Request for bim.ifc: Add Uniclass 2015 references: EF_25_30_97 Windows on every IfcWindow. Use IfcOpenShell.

First a look at what the model holds.

```python
import ifcopenshell

model = ifcopenshell.open("bim.ifc")
print(model.schema)
print("classifications:", [c.Name for c in model.by_type("IfcClassification")])
for ifc_class in ("IfcDoor", "IfcRoof", "IfcStair", "IfcWall", "IfcWindow"):
    print(ifc_class, len(model.by_type(ifc_class)))
```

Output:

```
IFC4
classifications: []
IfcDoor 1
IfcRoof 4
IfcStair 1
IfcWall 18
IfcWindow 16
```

```python
import ifcopenshell
import ifcopenshell.api.classification

model = ifcopenshell.open("bim.ifc")

system = ifcopenshell.api.classification.add_classification(model, classification="Uniclass 2015")

codes = {
    "IfcWindow": ("EF_25_30_97", "Windows"),
}
for ifc_class, (code, name) in codes.items():
    products = model.by_type(ifc_class)
    ifcopenshell.api.classification.add_reference(
        model, products=products, classification=system, identification=code, name=name
    )
    print(code, len(products))

model.write("bim_rev.ifc")
```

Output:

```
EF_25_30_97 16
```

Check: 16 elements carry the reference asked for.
